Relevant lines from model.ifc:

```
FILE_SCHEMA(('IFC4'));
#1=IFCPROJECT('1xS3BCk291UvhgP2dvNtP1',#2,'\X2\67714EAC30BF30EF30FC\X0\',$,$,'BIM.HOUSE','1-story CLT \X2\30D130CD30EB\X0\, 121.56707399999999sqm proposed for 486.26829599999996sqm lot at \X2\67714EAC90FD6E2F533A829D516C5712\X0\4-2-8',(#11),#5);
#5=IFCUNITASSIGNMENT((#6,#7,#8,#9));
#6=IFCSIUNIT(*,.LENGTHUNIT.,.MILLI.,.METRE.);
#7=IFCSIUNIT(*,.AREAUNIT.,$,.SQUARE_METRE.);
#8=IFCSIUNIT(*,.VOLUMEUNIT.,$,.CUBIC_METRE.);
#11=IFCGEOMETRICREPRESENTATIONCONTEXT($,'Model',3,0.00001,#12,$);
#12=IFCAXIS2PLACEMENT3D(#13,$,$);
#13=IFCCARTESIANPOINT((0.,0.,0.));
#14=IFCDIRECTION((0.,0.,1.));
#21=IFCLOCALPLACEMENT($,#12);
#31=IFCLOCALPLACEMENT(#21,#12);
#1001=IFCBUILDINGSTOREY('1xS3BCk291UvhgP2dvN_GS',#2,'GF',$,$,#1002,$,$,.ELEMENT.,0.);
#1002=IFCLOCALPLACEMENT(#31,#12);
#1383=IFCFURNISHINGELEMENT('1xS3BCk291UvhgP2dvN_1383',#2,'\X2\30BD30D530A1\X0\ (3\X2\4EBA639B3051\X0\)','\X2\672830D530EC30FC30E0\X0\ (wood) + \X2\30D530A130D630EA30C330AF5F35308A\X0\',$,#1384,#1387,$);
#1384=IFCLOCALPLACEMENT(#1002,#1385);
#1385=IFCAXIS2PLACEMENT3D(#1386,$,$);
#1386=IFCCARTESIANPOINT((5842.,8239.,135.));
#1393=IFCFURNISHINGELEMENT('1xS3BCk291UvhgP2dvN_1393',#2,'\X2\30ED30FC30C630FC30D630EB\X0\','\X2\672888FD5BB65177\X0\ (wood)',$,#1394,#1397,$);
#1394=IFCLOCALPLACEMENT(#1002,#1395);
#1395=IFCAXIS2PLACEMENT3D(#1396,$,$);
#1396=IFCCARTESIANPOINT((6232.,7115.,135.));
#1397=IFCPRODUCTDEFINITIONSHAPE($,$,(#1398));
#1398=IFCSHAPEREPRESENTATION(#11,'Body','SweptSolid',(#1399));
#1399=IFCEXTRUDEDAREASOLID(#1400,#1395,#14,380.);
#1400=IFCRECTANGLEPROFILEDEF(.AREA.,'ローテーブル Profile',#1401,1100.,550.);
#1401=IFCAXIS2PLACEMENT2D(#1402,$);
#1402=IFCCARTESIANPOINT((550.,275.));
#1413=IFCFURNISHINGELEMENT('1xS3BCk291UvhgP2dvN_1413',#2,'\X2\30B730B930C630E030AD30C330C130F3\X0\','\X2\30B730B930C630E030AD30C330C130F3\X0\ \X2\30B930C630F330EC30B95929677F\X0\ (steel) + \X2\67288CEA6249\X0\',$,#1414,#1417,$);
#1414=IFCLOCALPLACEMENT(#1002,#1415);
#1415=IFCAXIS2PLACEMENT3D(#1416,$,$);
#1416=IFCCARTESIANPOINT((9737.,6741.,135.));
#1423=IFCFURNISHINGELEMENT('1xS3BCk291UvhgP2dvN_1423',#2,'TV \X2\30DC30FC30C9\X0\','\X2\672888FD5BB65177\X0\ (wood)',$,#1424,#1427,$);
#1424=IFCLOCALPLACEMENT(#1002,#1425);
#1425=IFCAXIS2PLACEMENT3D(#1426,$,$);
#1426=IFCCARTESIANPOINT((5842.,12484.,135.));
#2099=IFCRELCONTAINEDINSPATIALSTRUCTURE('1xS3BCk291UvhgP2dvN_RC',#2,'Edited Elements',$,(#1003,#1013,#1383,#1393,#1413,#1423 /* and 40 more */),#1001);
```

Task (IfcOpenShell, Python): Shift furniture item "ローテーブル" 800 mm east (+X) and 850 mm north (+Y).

```python
import ifcopenshell
import ifcopenshell.api.geometry
import ifcopenshell.util.placement

model = ifcopenshell.open("model.ifc")

item = model.by_guid("1xS3BCk291UvhgP2dvN_1393")
matrix = ifcopenshell.util.placement.get_local_placement(item.ObjectPlacement)
matrix[0, 3] += 800.0
matrix[1, 3] += 850.0
ifcopenshell.api.geometry.edit_object_placement(model, product=item, matrix=matrix, is_si=False)

print(ifcopenshell.util.placement.get_local_placement(item.ObjectPlacement).round(3) + 0.0)

model.write("model_v2.ifc")
```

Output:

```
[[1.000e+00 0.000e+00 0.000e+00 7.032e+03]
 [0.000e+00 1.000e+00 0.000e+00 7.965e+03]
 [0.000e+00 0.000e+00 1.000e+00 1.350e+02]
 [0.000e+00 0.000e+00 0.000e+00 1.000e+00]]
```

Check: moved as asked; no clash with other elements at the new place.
